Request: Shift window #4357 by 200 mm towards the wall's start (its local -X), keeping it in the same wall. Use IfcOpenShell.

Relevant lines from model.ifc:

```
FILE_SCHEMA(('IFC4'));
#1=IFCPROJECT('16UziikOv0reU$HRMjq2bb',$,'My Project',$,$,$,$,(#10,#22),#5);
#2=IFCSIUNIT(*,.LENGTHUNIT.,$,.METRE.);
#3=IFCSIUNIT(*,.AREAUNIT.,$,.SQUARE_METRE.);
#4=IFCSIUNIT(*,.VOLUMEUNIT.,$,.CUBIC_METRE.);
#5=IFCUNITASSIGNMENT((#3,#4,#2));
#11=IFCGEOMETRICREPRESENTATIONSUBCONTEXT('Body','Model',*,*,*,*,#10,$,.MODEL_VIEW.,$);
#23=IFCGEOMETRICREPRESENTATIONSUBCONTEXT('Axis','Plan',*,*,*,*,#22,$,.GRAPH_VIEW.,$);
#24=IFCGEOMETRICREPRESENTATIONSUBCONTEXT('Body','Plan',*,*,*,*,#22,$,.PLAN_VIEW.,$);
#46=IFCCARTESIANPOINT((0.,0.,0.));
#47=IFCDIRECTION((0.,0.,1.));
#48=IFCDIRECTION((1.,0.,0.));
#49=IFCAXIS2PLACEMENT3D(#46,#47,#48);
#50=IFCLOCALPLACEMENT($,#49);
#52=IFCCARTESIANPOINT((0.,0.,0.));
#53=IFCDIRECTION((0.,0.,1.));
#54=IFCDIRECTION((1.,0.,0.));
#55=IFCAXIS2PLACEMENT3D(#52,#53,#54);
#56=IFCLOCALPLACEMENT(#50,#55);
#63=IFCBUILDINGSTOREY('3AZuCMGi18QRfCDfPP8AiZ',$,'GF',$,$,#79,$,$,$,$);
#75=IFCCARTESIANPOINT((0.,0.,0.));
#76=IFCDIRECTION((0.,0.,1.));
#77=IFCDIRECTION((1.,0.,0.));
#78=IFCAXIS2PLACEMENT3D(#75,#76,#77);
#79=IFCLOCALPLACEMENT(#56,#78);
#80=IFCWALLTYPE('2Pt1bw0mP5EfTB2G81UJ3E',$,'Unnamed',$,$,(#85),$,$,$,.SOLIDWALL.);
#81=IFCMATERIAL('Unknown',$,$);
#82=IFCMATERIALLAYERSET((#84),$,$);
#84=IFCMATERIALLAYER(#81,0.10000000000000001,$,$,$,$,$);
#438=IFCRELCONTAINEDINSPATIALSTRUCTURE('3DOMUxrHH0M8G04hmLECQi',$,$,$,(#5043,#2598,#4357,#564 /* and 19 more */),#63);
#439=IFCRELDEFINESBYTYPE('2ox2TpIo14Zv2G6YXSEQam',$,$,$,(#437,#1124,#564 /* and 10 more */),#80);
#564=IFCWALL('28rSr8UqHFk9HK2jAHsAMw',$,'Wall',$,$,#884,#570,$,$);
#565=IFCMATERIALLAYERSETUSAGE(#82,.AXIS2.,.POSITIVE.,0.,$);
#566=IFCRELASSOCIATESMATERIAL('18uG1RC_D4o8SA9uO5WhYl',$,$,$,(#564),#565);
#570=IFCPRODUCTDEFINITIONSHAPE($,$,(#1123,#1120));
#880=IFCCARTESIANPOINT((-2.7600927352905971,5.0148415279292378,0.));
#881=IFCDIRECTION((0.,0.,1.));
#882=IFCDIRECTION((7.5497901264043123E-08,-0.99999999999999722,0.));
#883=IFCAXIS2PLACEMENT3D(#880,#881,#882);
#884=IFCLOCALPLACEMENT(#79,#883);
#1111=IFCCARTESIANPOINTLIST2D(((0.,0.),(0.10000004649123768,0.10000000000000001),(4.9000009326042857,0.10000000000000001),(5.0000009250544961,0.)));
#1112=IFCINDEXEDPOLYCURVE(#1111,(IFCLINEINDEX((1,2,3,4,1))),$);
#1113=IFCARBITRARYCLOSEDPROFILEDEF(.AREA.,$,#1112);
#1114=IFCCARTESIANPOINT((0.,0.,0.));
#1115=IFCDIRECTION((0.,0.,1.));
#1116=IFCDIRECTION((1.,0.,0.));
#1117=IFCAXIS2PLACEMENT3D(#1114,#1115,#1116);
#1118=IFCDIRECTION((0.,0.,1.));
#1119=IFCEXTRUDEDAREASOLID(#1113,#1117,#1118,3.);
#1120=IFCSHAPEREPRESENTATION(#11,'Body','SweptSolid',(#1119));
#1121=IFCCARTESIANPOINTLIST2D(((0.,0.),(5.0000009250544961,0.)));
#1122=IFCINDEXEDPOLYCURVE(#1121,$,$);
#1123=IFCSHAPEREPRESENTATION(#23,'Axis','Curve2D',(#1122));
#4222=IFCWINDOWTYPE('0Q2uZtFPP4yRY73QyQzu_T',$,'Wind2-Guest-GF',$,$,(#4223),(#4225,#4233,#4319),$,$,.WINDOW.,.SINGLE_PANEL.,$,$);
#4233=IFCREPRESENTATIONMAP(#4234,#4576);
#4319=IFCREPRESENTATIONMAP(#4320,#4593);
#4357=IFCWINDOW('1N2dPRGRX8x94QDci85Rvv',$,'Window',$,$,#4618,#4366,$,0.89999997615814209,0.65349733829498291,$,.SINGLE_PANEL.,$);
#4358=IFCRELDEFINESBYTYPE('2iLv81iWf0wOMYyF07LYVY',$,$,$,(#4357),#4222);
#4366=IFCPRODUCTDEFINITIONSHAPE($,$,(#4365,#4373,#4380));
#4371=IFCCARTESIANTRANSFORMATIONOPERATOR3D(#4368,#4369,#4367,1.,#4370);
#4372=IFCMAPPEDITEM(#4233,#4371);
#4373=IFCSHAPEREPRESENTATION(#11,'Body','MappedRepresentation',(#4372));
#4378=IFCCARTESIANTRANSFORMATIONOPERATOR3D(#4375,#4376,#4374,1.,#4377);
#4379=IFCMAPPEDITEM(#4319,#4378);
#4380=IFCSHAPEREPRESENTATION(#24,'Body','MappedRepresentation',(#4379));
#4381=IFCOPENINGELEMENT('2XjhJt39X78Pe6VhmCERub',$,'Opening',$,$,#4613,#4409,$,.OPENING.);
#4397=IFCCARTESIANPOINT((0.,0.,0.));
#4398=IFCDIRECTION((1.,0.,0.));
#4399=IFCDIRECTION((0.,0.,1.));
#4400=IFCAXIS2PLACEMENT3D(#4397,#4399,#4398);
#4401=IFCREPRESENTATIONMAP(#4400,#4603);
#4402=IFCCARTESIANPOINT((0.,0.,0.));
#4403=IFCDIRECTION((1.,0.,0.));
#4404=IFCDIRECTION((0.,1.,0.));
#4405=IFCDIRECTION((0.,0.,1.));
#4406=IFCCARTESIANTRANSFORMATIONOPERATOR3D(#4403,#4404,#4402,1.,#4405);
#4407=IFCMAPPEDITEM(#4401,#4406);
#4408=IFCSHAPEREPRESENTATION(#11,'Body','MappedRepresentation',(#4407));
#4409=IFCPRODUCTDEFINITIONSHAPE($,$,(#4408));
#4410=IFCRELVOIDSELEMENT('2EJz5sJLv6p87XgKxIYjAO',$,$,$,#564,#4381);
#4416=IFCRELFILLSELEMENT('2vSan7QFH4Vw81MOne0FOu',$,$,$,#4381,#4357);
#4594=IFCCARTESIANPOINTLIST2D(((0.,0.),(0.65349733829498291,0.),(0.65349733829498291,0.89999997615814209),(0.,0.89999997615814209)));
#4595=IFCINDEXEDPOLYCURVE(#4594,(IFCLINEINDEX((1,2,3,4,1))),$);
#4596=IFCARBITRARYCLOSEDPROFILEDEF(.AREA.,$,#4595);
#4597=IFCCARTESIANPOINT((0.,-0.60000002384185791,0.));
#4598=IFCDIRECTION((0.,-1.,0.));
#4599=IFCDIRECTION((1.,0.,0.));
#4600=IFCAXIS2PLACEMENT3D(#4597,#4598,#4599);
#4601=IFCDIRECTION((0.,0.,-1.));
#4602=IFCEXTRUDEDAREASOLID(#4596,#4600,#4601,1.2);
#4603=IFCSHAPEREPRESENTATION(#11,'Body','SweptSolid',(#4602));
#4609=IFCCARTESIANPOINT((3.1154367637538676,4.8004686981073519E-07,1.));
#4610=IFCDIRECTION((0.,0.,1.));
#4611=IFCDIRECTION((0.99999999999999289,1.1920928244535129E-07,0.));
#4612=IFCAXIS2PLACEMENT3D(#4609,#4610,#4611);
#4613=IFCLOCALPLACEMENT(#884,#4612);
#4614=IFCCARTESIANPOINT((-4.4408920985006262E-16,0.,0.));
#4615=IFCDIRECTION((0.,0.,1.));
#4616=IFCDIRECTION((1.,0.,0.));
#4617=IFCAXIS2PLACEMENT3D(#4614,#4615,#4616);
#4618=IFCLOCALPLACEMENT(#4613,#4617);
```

```python
import ifcopenshell
import ifcopenshell.api.geometry
import ifcopenshell.util.placement
import ifcopenshell.util.unit

model = ifcopenshell.open("model.ifc")
unit_scale = ifcopenshell.util.unit.calculate_unit_scale(model)

window = model.by_guid("1N2dPRGRX8x94QDci85Rvv")
opening = window.FillsVoids[0].RelatingOpeningElement
wall = opening.VoidsElements[0].RelatingBuildingElement

wall_matrix = ifcopenshell.util.placement.get_local_placement(wall.ObjectPlacement)
shift = wall_matrix[:3, 0] * -0.2 / unit_scale
before = ifcopenshell.util.placement.get_local_placement(window.ObjectPlacement)[:3, 3].copy()

# The window is placed relative to its opening, so it follows when the opening moves.
matrix = ifcopenshell.util.placement.get_local_placement(opening.ObjectPlacement)
matrix[:3, 3] += shift
ifcopenshell.api.geometry.edit_object_placement(
    model, product=opening, matrix=matrix, is_si=False, should_transform_children=True
)

after = ifcopenshell.util.placement.get_local_placement(window.ObjectPlacement)[:3, 3]
print("window moved by", (after - before).round(3) + 0.0)

model.write("model_v2.ifc")
```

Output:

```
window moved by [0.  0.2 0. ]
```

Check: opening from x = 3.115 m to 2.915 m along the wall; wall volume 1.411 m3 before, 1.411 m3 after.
